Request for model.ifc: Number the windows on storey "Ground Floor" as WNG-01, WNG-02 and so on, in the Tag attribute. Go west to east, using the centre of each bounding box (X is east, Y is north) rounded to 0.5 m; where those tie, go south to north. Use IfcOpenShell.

First a look at what the model holds.

```python
import ifcopenshell
import ifcopenshell.util.element
import ifcopenshell.util.placement

model = ifcopenshell.open("model.ifc")
print(model.schema)
storey = next(s for s in model.by_type("IfcBuildingStorey") if s.Name == "Ground Floor")
windows = [e for e in ifcopenshell.util.element.get_decomposition(storey) if e.is_a("IfcWindow")]
for e in sorted(windows, key=lambda e: e.id()):
    origin = ifcopenshell.util.placement.get_local_placement(e.ObjectPlacement)[:3, 3]
    print(e.id(), e.Tag, e.Name, origin.round(2) + 0.0, sep=" | ")
```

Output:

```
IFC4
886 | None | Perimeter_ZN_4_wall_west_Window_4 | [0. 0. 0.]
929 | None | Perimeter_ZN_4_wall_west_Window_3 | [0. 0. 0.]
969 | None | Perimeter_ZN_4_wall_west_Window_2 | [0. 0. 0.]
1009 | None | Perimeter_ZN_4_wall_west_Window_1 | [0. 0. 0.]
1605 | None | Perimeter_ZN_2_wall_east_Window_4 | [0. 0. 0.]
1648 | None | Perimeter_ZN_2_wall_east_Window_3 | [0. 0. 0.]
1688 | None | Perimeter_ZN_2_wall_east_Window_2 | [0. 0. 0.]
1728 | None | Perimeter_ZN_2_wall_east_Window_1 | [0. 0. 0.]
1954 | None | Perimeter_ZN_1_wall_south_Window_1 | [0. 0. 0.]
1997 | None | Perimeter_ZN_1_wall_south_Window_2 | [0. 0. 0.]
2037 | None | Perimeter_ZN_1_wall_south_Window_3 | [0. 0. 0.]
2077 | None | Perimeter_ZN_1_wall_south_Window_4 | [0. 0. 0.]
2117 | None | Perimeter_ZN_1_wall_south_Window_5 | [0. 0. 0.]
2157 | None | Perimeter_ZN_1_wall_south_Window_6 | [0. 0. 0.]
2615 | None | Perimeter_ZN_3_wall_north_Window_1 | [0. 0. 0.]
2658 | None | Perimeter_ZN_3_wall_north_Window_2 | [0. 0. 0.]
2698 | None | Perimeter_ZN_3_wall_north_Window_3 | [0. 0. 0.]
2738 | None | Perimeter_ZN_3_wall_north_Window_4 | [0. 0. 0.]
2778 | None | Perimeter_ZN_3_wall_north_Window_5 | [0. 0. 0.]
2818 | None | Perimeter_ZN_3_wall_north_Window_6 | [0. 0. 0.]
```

```python
import ifcopenshell
import ifcopenshell.geom
import ifcopenshell.util.element
import ifcopenshell.util.shape

model = ifcopenshell.open("model.ifc")
settings = ifcopenshell.geom.settings()
settings.set("use-world-coords", True)


def centre(element):
    shape = ifcopenshell.geom.create_shape(settings, element)
    return ifcopenshell.util.shape.get_bbox_centroid(shape.geometry)


storey = next(s for s in model.by_type("IfcBuildingStorey") if s.Name == "Ground Floor")
windows = [e for e in ifcopenshell.util.element.get_decomposition(storey) if e.is_a("IfcWindow")]

# Insertion points can sit at a corner or the storey origin, so sort by the geometry (in metres).
centres = {e: centre(e) for e in windows}
windows.sort(key=lambda e: (round(centres[e][0] / 0.5), centres[e][1]))

for i, e in enumerate(windows, start=1):
    number = f"WNG-{i:02d}"
    e.Tag = number
    print(e.id(), number)

model.write("model_edited.ifc")
```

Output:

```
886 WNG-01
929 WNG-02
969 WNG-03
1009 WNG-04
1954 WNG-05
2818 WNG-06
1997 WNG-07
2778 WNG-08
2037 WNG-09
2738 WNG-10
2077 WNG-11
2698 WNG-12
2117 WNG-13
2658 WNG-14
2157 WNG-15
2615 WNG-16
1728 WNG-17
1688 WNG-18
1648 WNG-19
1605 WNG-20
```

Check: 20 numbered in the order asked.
